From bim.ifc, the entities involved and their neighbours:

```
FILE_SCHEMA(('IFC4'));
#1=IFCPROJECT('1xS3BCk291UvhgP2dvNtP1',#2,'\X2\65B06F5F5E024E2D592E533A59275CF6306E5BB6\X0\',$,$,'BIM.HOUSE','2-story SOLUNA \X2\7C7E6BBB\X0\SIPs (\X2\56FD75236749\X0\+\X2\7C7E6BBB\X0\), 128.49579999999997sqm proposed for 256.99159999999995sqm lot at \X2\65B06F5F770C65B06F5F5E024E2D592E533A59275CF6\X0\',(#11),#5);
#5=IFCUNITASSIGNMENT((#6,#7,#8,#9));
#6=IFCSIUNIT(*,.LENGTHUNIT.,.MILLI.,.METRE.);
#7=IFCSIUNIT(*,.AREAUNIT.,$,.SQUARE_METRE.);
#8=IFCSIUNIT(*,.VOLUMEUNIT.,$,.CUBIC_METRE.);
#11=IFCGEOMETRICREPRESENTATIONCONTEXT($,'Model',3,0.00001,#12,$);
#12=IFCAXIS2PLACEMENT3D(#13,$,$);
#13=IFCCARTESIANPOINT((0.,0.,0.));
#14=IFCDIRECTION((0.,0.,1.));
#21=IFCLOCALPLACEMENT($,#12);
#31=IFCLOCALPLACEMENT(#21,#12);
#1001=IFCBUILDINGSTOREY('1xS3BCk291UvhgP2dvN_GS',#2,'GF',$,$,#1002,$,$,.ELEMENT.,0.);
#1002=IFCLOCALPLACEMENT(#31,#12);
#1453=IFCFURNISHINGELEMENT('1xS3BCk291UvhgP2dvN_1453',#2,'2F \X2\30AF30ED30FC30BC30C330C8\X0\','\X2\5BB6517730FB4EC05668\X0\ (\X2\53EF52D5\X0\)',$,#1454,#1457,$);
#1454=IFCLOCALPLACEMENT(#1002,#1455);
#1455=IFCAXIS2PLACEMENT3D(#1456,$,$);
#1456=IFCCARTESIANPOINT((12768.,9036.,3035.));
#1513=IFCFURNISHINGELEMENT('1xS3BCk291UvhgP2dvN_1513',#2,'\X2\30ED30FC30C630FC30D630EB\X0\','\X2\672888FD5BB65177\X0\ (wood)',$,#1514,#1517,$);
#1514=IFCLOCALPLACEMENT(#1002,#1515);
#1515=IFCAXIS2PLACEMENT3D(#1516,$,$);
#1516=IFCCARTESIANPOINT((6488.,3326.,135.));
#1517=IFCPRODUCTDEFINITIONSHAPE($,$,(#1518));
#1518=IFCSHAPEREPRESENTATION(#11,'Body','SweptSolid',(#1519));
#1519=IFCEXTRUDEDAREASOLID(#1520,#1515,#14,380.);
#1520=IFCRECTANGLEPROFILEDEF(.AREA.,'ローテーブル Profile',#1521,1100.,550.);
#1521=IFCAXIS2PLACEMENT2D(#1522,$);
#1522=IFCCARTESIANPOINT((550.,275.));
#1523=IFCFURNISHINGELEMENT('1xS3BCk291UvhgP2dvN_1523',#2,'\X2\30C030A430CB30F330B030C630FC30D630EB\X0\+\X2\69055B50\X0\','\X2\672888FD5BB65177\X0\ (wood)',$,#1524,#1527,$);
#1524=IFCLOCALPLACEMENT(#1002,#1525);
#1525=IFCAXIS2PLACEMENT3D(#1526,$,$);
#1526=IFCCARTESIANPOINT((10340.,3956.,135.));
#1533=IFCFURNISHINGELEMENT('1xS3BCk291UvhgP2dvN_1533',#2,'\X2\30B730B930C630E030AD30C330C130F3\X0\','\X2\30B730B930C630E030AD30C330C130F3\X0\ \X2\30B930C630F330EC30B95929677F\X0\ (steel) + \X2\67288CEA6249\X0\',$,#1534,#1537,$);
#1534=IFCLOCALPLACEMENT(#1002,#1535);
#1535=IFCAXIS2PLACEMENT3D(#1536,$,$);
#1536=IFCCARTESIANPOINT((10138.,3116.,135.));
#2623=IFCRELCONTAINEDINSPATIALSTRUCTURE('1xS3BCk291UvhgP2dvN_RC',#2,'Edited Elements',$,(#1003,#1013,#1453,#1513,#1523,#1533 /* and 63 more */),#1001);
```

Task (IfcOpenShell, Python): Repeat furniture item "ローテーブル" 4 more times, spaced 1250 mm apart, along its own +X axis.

```python
import ifcopenshell
import ifcopenshell.api.geometry
import ifcopenshell.api.root
import ifcopenshell.util.element
import ifcopenshell.util.placement
import ifcopenshell.util.unit

model = ifcopenshell.open("bim.ifc")
unit_scale = ifcopenshell.util.unit.calculate_unit_scale(model)


def reuse_history(source, copy):
    """copy_class also copies each property set's owner history, people and application; keep the originals."""
    for rel in copy.IsDefinedBy:
        if rel.is_a("IfcRelDefinesByProperties") and (history := rel.RelatingPropertyDefinition.OwnerHistory):
            rel.RelatingPropertyDefinition.OwnerHistory = source.OwnerHistory
            ifcopenshell.util.element.remove_deep2(model, history)


source = model.by_id(1513)
base = ifcopenshell.util.placement.get_local_placement(source.ObjectPlacement)
step = base[:3, 0] * 1.25 / unit_scale

for i in range(1, 5):
    copy = ifcopenshell.api.root.copy_class(model, product=source)
    copy.Representation = ifcopenshell.util.element.copy_deep(
        model, source.Representation, exclude=["IfcGeometricRepresentationContext", "IfcRepresentationMap"]
    )
    reuse_history(source, copy)
    matrix = base.copy()
    matrix[:3, 3] += i * step
    print("added at", matrix[:3, 3].round(3) + 0.0)
    ifcopenshell.api.geometry.edit_object_placement(model, product=copy, matrix=matrix, is_si=False)

model.write("bim_updated.ifc")
```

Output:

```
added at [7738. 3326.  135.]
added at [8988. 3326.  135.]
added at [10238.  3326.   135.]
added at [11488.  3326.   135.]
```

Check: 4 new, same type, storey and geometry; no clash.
